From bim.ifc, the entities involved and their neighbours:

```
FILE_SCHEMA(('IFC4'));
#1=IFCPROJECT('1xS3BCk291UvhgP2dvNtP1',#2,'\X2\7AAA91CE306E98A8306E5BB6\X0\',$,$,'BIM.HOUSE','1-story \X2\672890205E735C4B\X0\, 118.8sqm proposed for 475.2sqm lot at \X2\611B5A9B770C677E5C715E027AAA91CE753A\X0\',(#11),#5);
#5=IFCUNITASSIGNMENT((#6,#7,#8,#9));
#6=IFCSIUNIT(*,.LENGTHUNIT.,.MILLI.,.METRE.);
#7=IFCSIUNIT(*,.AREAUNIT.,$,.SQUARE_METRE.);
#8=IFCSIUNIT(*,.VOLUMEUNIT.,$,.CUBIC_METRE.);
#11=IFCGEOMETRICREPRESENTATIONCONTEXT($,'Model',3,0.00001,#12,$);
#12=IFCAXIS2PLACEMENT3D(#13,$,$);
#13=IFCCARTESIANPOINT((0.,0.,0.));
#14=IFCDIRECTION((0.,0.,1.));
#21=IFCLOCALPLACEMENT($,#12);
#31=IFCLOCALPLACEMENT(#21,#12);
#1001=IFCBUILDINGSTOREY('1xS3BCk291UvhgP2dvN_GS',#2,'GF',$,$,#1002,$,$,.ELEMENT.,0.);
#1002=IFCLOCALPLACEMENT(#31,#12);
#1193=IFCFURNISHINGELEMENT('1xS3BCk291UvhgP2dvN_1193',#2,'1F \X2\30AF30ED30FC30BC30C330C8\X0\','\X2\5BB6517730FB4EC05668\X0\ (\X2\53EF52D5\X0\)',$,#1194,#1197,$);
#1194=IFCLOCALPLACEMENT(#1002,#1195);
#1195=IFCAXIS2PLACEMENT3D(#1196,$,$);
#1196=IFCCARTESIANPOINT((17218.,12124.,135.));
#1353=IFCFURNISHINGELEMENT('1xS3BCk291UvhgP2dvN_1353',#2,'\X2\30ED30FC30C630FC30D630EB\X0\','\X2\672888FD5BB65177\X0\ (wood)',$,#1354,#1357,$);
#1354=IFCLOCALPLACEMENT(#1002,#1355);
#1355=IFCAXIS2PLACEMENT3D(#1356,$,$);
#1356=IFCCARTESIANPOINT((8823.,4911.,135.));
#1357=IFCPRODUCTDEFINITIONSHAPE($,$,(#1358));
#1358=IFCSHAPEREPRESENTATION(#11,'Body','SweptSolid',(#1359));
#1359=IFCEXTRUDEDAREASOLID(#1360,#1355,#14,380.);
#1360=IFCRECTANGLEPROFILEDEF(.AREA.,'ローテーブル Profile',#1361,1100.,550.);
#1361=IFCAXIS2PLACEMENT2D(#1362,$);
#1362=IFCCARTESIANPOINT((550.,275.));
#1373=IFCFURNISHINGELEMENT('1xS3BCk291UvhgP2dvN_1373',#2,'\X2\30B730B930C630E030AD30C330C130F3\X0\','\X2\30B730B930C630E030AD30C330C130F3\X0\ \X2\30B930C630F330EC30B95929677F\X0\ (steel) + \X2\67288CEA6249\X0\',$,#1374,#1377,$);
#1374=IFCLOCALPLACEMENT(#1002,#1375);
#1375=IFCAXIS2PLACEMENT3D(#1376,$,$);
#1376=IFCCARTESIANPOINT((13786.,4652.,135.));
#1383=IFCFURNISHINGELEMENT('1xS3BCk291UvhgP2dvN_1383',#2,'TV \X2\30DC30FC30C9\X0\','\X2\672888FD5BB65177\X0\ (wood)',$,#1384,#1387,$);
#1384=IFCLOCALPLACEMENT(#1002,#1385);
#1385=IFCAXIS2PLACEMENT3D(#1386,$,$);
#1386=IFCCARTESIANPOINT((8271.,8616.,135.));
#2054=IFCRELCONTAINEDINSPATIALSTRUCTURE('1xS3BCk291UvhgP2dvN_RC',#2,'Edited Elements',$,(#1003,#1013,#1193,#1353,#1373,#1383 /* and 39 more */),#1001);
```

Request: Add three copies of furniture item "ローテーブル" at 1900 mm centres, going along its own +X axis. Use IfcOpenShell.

```python
import ifcopenshell
import ifcopenshell.api.geometry
import ifcopenshell.api.root
import ifcopenshell.util.element
import ifcopenshell.util.placement
import ifcopenshell.util.unit

model = ifcopenshell.open("bim.ifc")
unit_scale = ifcopenshell.util.unit.calculate_unit_scale(model)


def reuse_history(source, copy):
    """copy_class also copies each property set's owner history, people and application; keep the originals."""
    for rel in copy.IsDefinedBy:
        if rel.is_a("IfcRelDefinesByProperties") and (history := rel.RelatingPropertyDefinition.OwnerHistory):
            rel.RelatingPropertyDefinition.OwnerHistory = source.OwnerHistory
            ifcopenshell.util.element.remove_deep2(model, history)


source = model.by_guid("1xS3BCk291UvhgP2dvN_1353")
base = ifcopenshell.util.placement.get_local_placement(source.ObjectPlacement)
step = base[:3, 0] * 1.9 / unit_scale

for i in range(1, 4):
    copy = ifcopenshell.api.root.copy_class(model, product=source)
    copy.Representation = ifcopenshell.util.element.copy_deep(
        model, source.Representation, exclude=["IfcGeometricRepresentationContext", "IfcRepresentationMap"]
    )
    reuse_history(source, copy)
    matrix = base.copy()
    matrix[:3, 3] += i * step
    print("added at", matrix[:3, 3].round(3) + 0.0)
    ifcopenshell.api.geometry.edit_object_placement(model, product=copy, matrix=matrix, is_si=False)

model.write("bim_updated.ifc")
```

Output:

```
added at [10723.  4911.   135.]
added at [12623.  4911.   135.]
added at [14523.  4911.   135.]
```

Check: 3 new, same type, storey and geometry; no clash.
